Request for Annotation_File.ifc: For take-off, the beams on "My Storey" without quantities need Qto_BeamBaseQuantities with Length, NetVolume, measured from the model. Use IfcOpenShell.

First a look at what the model holds.

```python
import ifcopenshell
import ifcopenshell.util.element
import ifcopenshell.util.unit

model = ifcopenshell.open("Annotation_File.ifc")
print(model.schema)
for unit_type in ("LENGTHUNIT", "AREAUNIT", "VOLUMEUNIT"):
    print(unit_type, ifcopenshell.util.unit.calculate_unit_scale(model, unit_type))
storey = next(s for s in model.by_type("IfcBuildingStorey") if s.Name == "My Storey")
beams = [e for e in ifcopenshell.util.element.get_decomposition(storey) if e.is_a("IfcBeam")]
for e in sorted(beams, key=lambda e: e.id()):
    print(e.id(), e.is_a(), e.Name, list(ifcopenshell.util.element.get_psets(e, qtos_only=True)), sep=" | ")
```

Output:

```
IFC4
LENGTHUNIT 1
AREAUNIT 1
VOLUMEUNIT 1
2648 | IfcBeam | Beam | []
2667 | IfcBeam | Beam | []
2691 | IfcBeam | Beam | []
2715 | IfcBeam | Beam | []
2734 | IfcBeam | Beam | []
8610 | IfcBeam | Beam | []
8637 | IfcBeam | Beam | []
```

```python
import ifcopenshell
import ifcopenshell.api.pset
import ifcopenshell.geom
import ifcopenshell.util.element
import ifcopenshell.util.shape
import ifcopenshell.util.unit

model = ifcopenshell.open("Annotation_File.ifc")
unit_scale = ifcopenshell.util.unit.calculate_unit_scale(model)
volume_scale = ifcopenshell.util.unit.calculate_unit_scale(model, "VOLUMEUNIT")
settings = ifcopenshell.geom.settings()

storey = next(s for s in model.by_type("IfcBuildingStorey") if s.Name == "My Storey")
beams = [e for e in ifcopenshell.util.element.get_decomposition(storey) if e.is_a("IfcBeam")]

for e in sorted(beams, key=lambda e: e.id()):
    if ifcopenshell.util.element.get_psets(e, qtos_only=True, should_inherit=False):
        continue
    # Geometry comes back in metres, in the element's own axes.
    shape = ifcopenshell.geom.create_shape(settings, e)
    values = {
        "Length": ifcopenshell.util.shape.get_max_xyz(shape.geometry) / unit_scale,
        "NetVolume": ifcopenshell.util.shape.get_volume(shape.geometry) / volume_scale,
    }
    qto = ifcopenshell.api.pset.add_qto(model, product=e, name="Qto_BeamBaseQuantities")
    ifcopenshell.api.pset.edit_qto(model, qto=qto, properties=values)
    print(e.id(), {k: round(v, 3) for k, v in values.items()})

model.write("Annotation_File_updated.ifc")
```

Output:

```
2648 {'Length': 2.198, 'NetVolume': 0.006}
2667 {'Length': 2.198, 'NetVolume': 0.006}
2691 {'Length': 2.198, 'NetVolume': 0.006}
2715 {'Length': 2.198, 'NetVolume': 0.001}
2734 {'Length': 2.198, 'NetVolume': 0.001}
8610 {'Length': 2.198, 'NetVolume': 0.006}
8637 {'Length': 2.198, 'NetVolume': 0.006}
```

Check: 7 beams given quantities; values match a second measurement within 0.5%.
